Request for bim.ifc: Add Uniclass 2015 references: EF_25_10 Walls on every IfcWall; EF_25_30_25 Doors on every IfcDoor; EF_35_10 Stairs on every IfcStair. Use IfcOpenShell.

First a look at what the model holds.

```python
import ifcopenshell

model = ifcopenshell.open("bim.ifc")
print(model.schema)
print("classifications:", [c.Name for c in model.by_type("IfcClassification")])
for ifc_class in ("IfcDoor", "IfcRoof", "IfcStair", "IfcWall", "IfcWindow"):
    print(ifc_class, len(model.by_type(ifc_class)))
```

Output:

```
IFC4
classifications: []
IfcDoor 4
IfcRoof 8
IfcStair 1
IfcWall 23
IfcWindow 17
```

```python
import ifcopenshell
import ifcopenshell.api.classification

model = ifcopenshell.open("bim.ifc")

system = ifcopenshell.api.classification.add_classification(model, classification="Uniclass 2015")

codes = {
    "IfcWall": ("EF_25_10", "Walls"),
    "IfcDoor": ("EF_25_30_25", "Doors"),
    "IfcStair": ("EF_35_10", "Stairs"),
}
for ifc_class, (code, name) in codes.items():
    products = model.by_type(ifc_class)
    ifcopenshell.api.classification.add_reference(
        model, products=products, classification=system, identification=code, name=name
    )
    print(code, len(products))

model.write("bim_edited.ifc")
```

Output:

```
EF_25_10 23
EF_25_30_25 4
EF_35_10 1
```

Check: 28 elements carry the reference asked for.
